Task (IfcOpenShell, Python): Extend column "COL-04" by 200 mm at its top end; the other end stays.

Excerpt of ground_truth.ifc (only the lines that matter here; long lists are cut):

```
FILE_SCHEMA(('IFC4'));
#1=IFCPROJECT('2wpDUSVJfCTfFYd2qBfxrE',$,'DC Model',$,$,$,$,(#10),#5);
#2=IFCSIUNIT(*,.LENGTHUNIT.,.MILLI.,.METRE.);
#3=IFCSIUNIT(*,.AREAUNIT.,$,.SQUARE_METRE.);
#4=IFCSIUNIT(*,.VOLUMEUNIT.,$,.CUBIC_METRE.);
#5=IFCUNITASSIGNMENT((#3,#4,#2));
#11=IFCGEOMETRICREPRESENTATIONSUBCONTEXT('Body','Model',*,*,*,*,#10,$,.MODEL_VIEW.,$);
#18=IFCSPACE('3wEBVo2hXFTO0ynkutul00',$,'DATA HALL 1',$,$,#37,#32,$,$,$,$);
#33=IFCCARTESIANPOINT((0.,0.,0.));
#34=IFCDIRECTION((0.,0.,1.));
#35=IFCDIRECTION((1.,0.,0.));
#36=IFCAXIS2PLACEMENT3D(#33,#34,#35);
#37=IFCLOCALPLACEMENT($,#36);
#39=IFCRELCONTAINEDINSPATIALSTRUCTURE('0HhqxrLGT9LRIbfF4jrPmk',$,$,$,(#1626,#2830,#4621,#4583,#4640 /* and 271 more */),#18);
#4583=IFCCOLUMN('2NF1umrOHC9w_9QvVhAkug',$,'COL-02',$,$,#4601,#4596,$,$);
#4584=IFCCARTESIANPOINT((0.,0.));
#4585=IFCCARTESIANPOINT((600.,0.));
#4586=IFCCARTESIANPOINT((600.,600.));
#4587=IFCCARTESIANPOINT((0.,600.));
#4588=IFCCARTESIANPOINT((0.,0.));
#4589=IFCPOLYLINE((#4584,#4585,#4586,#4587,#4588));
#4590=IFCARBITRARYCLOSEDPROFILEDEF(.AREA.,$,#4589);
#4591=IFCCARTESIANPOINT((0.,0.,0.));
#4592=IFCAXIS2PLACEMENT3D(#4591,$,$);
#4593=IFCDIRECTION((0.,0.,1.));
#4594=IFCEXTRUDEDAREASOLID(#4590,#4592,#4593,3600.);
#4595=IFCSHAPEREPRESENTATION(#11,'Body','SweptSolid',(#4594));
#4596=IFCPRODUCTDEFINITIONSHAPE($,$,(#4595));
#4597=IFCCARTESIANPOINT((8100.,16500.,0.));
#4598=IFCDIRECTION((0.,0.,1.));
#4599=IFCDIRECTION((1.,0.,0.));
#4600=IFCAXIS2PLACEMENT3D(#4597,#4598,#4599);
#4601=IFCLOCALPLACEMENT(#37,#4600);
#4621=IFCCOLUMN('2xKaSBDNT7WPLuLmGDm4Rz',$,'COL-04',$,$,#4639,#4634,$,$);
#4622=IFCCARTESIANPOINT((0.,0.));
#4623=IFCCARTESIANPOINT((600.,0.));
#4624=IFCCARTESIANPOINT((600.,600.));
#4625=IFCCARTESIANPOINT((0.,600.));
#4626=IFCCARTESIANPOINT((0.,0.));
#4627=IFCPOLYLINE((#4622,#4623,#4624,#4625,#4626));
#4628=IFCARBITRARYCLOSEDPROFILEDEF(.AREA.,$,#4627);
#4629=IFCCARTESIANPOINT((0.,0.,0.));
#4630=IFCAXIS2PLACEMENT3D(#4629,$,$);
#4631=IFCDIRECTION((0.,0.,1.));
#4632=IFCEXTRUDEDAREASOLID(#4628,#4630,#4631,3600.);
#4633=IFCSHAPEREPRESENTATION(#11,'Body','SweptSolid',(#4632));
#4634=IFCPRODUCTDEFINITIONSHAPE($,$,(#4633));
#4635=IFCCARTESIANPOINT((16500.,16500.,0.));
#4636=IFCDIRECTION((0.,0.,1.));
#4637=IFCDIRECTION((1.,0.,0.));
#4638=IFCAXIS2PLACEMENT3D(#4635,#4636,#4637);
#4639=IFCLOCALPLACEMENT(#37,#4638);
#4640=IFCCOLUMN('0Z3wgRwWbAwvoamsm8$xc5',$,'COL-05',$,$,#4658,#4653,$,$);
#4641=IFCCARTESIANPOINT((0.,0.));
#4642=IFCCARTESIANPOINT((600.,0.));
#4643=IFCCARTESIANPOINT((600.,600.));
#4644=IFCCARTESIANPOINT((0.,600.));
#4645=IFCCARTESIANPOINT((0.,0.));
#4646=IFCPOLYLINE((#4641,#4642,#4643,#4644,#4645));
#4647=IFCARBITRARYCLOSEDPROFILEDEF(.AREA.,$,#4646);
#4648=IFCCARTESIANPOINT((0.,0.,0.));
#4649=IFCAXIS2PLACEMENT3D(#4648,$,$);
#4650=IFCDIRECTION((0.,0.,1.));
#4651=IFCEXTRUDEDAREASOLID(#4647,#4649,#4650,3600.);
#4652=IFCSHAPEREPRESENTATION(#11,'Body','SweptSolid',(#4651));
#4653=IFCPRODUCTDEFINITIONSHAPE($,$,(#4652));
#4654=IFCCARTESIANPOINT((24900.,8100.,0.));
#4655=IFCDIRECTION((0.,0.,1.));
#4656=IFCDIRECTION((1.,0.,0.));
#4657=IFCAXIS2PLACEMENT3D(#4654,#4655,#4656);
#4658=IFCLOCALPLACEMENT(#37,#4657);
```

```python
import ifcopenshell
import ifcopenshell.util.representation
import ifcopenshell.util.unit

model = ifcopenshell.open("ground_truth.ifc")
unit_scale = ifcopenshell.util.unit.calculate_unit_scale(model)

member = model.by_guid("2xKaSBDNT7WPLuLmGDm4Rz")
change = 0.2 / unit_scale

# The extrusion runs towards the end named, so only its depth changes.
body = ifcopenshell.util.representation.get_representation(member, "Model", "Body")
solid = body.Items[0]
old_length = solid.Depth
solid.Depth += change

print(f"length {old_length:g} -> {solid.Depth:g}")

model.write("ground_truth_rev.ifc")
```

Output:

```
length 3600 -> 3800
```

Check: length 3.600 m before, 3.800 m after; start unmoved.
